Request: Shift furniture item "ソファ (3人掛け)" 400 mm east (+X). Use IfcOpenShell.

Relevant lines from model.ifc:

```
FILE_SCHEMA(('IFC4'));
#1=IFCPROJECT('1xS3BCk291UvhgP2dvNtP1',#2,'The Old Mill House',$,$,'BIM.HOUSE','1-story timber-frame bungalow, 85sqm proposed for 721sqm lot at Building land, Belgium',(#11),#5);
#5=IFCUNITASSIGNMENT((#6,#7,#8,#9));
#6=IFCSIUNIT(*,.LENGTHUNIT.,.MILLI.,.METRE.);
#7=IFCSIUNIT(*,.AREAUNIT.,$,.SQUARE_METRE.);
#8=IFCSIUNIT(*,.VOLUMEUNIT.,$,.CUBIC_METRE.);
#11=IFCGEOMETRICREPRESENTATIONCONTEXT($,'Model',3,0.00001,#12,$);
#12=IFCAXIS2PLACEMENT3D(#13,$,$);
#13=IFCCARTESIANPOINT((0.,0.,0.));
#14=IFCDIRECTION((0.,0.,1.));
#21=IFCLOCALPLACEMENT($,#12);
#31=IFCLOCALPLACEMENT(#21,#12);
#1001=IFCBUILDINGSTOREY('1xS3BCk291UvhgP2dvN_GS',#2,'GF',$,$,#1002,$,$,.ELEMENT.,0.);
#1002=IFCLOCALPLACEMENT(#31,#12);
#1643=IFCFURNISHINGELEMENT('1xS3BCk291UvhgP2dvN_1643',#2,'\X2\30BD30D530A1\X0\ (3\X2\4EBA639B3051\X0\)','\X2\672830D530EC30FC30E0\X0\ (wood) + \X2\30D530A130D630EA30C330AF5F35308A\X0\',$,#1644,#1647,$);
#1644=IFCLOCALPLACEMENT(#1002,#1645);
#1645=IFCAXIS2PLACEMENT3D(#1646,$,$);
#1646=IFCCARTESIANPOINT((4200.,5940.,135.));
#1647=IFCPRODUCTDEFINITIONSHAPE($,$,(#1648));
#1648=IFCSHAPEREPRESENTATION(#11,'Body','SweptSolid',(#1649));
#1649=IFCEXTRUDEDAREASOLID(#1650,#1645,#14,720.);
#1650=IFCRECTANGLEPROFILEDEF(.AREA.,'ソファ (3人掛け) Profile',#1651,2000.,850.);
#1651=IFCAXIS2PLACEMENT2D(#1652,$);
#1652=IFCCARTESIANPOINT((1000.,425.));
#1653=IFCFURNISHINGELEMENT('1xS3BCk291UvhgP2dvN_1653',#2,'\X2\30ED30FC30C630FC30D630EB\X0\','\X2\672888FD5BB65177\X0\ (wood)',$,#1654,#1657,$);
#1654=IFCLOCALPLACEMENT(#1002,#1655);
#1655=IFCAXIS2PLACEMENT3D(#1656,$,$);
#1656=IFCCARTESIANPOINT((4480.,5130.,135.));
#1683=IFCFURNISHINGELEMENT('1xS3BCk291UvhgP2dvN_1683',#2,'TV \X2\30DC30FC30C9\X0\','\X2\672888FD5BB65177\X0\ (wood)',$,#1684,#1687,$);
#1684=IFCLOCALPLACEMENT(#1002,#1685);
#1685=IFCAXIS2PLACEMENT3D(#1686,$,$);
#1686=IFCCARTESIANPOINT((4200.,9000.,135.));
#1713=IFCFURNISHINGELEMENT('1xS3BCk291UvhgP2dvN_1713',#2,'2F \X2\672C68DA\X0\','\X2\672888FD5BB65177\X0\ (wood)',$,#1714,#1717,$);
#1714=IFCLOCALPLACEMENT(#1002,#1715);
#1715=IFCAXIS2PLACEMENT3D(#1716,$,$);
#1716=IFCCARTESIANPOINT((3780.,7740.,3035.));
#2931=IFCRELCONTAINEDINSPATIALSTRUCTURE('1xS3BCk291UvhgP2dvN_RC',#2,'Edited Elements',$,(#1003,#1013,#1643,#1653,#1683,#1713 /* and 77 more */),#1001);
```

```python
import ifcopenshell
import ifcopenshell.api.geometry
import ifcopenshell.util.placement
import ifcopenshell.util.unit

model = ifcopenshell.open("model.ifc")
unit_scale = ifcopenshell.util.unit.calculate_unit_scale(model)

item = model.by_guid("1xS3BCk291UvhgP2dvN_1643")
matrix = ifcopenshell.util.placement.get_local_placement(item.ObjectPlacement)
matrix[0, 3] += 0.4 / unit_scale
ifcopenshell.api.geometry.edit_object_placement(model, product=item, matrix=matrix, is_si=False)

print(ifcopenshell.util.placement.get_local_placement(item.ObjectPlacement).round(3) + 0.0)

model.write("model_v2.ifc")
```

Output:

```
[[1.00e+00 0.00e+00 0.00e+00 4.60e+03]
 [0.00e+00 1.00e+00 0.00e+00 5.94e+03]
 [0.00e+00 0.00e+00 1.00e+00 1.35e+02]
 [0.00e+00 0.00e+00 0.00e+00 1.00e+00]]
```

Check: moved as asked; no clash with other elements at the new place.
